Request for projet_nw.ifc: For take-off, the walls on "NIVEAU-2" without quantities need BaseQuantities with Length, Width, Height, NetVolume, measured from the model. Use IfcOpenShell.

First a look at what the model holds.

```python
import ifcopenshell
import ifcopenshell.util.element
import ifcopenshell.util.unit

model = ifcopenshell.open("projet_nw.ifc")
print(model.schema)
for unit_type in ("LENGTHUNIT", "AREAUNIT", "VOLUMEUNIT"):
    print(unit_type, ifcopenshell.util.unit.calculate_unit_scale(model, unit_type))
storey = next(s for s in model.by_type("IfcBuildingStorey") if s.Name == "NIVEAU-2")
walls = [e for e in ifcopenshell.util.element.get_decomposition(storey) if e.is_a("IfcWall")]
for e in sorted(walls, key=lambda e: e.id()):
    print(e.id(), e.is_a(), e.Name, list(ifcopenshell.util.element.get_psets(e, qtos_only=True)), sep=" | ")
```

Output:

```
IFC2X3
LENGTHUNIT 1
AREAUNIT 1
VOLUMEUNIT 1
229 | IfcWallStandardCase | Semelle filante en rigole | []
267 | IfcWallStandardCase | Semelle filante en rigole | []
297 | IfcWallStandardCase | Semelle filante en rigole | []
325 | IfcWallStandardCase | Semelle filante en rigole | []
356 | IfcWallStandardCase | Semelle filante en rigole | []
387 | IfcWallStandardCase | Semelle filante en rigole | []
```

```python
import ifcopenshell
import ifcopenshell.api.pset
import ifcopenshell.geom
import ifcopenshell.util.element
import ifcopenshell.util.shape
import ifcopenshell.util.unit

model = ifcopenshell.open("projet_nw.ifc")
unit_scale = ifcopenshell.util.unit.calculate_unit_scale(model)
volume_scale = ifcopenshell.util.unit.calculate_unit_scale(model, "VOLUMEUNIT")
settings = ifcopenshell.geom.settings()

storey = next(s for s in model.by_type("IfcBuildingStorey") if s.Name == "NIVEAU-2")
walls = [e for e in ifcopenshell.util.element.get_decomposition(storey) if e.is_a("IfcWall")]

for e in sorted(walls, key=lambda e: e.id()):
    if ifcopenshell.util.element.get_psets(e, qtos_only=True, should_inherit=False):
        continue
    # Geometry comes back in metres, in the element's own axes.
    shape = ifcopenshell.geom.create_shape(settings, e)
    values = {
        "Length": ifcopenshell.util.shape.get_x(shape.geometry) / unit_scale,
        "Width": ifcopenshell.util.shape.get_y(shape.geometry) / unit_scale,
        "Height": ifcopenshell.util.shape.get_z(shape.geometry) / unit_scale,
        "NetVolume": ifcopenshell.util.shape.get_volume(shape.geometry) / volume_scale,
    }
    qto = ifcopenshell.api.pset.add_qto(model, product=e, name="BaseQuantities")
    ifcopenshell.api.pset.edit_qto(model, qto=qto, properties=values)
    print(e.id(), {k: round(v, 3) for k, v in values.items()})

model.write("projet_nw_updated.ifc")
```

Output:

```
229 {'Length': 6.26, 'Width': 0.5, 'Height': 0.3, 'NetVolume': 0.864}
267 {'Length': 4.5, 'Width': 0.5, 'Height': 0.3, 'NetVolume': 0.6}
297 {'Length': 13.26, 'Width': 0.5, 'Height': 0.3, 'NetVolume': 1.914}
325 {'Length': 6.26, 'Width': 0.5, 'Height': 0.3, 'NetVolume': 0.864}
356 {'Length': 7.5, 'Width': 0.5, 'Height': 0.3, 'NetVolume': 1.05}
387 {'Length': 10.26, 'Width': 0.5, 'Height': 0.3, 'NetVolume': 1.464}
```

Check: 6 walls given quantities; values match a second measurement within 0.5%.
